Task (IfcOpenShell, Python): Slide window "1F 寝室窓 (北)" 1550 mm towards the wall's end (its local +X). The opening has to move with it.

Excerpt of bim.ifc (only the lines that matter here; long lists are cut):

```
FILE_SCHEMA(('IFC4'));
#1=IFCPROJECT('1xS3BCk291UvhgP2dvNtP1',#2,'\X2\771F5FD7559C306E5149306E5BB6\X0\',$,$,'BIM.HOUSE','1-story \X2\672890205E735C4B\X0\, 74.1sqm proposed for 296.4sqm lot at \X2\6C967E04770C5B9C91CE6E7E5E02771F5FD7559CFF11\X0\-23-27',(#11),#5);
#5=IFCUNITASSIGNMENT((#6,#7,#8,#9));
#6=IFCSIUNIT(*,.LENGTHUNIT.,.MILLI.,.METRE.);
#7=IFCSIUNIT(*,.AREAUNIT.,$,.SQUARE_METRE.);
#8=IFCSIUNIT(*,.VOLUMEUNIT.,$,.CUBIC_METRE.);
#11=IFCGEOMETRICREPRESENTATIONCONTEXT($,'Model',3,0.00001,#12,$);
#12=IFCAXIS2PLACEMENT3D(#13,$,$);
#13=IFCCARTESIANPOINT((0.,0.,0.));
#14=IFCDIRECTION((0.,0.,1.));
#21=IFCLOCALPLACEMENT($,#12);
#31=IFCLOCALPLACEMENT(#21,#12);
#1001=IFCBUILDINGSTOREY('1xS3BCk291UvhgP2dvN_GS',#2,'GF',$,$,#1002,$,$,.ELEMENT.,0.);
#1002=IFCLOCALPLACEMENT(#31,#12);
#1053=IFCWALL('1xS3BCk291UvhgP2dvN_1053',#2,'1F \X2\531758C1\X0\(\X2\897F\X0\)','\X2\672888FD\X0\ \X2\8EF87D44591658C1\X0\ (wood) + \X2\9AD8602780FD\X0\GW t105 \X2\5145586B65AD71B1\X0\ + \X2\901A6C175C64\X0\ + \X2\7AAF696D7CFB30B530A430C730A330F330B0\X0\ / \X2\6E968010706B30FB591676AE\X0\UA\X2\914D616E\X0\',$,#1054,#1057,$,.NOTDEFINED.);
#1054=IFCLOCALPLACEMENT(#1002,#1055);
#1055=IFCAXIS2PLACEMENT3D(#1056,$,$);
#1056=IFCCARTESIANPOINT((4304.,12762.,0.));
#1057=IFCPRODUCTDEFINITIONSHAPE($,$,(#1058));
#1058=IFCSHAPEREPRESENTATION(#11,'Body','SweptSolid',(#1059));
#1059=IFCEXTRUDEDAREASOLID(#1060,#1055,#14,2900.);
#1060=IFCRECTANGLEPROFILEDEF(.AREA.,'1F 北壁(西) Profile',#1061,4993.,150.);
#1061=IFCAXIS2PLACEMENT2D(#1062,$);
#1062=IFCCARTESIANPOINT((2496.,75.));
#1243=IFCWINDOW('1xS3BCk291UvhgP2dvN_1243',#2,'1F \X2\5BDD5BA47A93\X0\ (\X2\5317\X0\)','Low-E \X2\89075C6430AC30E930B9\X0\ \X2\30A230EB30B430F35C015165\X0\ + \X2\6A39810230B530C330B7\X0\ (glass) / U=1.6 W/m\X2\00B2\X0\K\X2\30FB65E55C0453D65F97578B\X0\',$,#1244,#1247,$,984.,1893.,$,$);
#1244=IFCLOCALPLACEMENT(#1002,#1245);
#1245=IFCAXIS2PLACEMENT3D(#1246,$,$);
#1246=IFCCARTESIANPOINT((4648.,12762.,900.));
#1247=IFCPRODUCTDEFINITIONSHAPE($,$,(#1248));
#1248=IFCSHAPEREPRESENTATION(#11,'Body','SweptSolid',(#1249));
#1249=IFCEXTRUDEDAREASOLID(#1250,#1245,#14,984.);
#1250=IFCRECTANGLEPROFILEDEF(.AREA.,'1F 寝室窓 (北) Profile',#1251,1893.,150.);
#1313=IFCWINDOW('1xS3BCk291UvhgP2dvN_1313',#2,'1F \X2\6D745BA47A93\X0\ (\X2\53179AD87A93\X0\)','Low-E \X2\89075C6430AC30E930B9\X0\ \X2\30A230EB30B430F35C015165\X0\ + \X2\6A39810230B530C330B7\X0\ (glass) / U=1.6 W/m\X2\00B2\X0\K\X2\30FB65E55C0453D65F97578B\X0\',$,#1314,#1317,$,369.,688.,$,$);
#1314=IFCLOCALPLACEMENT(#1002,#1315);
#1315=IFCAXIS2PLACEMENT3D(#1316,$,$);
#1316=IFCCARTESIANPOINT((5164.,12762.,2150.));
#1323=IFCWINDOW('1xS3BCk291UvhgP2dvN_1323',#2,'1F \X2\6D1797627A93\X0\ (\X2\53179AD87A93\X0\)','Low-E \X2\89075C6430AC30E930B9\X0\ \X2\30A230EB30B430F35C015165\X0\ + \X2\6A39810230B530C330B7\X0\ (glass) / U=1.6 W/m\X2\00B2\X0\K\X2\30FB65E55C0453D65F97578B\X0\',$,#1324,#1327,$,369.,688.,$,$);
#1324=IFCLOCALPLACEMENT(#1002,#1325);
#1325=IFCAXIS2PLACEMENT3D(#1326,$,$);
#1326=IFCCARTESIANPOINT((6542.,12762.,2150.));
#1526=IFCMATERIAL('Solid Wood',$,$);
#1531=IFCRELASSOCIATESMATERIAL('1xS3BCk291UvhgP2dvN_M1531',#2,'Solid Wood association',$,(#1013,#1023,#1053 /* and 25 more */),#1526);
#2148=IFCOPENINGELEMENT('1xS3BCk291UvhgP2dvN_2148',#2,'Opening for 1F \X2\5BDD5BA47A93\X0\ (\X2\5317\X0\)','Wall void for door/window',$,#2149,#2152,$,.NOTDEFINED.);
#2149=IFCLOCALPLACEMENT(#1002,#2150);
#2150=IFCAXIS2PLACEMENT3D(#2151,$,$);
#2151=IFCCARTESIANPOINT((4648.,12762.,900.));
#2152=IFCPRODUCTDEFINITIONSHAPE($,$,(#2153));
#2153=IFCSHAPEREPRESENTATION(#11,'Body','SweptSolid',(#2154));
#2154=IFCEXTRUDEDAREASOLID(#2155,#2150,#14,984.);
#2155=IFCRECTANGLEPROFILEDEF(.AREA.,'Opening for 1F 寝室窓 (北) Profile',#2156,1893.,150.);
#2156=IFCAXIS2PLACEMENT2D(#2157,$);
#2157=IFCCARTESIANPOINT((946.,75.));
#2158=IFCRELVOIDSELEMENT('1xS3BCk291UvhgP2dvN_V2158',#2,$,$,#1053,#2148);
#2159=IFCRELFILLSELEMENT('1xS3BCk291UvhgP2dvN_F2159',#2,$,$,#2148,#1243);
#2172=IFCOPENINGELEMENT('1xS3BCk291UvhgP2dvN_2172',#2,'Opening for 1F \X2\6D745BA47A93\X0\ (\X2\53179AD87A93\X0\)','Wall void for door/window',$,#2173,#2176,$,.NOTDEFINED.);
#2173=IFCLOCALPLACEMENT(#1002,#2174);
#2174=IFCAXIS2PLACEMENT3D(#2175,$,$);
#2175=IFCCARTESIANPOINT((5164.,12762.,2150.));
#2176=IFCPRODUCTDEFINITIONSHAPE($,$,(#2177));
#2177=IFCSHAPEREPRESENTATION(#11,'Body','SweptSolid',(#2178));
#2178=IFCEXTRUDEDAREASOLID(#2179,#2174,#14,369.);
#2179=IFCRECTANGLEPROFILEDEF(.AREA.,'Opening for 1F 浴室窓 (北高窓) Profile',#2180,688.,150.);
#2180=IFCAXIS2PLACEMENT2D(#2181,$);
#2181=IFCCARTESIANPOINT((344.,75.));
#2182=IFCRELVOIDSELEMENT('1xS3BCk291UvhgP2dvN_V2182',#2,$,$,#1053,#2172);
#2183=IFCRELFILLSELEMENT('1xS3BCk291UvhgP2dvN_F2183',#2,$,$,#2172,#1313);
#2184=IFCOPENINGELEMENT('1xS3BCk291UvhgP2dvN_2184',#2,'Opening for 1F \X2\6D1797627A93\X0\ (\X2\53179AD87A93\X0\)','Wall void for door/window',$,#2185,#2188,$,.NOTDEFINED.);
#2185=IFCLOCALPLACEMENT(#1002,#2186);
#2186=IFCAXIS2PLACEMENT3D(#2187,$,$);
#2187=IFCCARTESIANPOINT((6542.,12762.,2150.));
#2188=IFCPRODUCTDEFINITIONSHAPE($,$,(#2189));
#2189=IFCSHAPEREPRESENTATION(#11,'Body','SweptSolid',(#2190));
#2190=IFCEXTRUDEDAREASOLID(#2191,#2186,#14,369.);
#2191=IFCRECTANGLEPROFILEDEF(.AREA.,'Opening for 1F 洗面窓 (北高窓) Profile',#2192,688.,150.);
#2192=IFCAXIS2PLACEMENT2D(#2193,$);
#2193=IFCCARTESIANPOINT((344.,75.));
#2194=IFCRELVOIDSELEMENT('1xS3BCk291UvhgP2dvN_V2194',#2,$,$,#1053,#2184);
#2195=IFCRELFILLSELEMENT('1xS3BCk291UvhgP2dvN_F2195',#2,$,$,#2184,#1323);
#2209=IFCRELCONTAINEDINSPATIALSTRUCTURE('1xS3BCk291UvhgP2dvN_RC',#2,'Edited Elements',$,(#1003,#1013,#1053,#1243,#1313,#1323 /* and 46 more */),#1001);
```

```python
import ifcopenshell
import ifcopenshell.api.geometry
import ifcopenshell.util.placement
import ifcopenshell.util.unit

model = ifcopenshell.open("bim.ifc")
unit_scale = ifcopenshell.util.unit.calculate_unit_scale(model)

window = model.by_guid("1xS3BCk291UvhgP2dvN_1243")
opening = window.FillsVoids[0].RelatingOpeningElement
wall = opening.VoidsElements[0].RelatingBuildingElement

wall_matrix = ifcopenshell.util.placement.get_local_placement(wall.ObjectPlacement)
shift = wall_matrix[:3, 0] * 1.55 / unit_scale
before = ifcopenshell.util.placement.get_local_placement(window.ObjectPlacement)[:3, 3].copy()

# The window is not placed relative to its opening, so move both.
for product in (opening, window):
    matrix = ifcopenshell.util.placement.get_local_placement(product.ObjectPlacement)
    matrix[:3, 3] += shift
    ifcopenshell.api.geometry.edit_object_placement(model, product=product, matrix=matrix, is_si=False)

after = ifcopenshell.util.placement.get_local_placement(window.ObjectPlacement)[:3, 3]
print("window moved by", (after - before).round(3) + 0.0)

model.write("bim_edited.ifc")
```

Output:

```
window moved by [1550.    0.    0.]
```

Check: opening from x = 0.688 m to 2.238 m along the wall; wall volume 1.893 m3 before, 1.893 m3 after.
